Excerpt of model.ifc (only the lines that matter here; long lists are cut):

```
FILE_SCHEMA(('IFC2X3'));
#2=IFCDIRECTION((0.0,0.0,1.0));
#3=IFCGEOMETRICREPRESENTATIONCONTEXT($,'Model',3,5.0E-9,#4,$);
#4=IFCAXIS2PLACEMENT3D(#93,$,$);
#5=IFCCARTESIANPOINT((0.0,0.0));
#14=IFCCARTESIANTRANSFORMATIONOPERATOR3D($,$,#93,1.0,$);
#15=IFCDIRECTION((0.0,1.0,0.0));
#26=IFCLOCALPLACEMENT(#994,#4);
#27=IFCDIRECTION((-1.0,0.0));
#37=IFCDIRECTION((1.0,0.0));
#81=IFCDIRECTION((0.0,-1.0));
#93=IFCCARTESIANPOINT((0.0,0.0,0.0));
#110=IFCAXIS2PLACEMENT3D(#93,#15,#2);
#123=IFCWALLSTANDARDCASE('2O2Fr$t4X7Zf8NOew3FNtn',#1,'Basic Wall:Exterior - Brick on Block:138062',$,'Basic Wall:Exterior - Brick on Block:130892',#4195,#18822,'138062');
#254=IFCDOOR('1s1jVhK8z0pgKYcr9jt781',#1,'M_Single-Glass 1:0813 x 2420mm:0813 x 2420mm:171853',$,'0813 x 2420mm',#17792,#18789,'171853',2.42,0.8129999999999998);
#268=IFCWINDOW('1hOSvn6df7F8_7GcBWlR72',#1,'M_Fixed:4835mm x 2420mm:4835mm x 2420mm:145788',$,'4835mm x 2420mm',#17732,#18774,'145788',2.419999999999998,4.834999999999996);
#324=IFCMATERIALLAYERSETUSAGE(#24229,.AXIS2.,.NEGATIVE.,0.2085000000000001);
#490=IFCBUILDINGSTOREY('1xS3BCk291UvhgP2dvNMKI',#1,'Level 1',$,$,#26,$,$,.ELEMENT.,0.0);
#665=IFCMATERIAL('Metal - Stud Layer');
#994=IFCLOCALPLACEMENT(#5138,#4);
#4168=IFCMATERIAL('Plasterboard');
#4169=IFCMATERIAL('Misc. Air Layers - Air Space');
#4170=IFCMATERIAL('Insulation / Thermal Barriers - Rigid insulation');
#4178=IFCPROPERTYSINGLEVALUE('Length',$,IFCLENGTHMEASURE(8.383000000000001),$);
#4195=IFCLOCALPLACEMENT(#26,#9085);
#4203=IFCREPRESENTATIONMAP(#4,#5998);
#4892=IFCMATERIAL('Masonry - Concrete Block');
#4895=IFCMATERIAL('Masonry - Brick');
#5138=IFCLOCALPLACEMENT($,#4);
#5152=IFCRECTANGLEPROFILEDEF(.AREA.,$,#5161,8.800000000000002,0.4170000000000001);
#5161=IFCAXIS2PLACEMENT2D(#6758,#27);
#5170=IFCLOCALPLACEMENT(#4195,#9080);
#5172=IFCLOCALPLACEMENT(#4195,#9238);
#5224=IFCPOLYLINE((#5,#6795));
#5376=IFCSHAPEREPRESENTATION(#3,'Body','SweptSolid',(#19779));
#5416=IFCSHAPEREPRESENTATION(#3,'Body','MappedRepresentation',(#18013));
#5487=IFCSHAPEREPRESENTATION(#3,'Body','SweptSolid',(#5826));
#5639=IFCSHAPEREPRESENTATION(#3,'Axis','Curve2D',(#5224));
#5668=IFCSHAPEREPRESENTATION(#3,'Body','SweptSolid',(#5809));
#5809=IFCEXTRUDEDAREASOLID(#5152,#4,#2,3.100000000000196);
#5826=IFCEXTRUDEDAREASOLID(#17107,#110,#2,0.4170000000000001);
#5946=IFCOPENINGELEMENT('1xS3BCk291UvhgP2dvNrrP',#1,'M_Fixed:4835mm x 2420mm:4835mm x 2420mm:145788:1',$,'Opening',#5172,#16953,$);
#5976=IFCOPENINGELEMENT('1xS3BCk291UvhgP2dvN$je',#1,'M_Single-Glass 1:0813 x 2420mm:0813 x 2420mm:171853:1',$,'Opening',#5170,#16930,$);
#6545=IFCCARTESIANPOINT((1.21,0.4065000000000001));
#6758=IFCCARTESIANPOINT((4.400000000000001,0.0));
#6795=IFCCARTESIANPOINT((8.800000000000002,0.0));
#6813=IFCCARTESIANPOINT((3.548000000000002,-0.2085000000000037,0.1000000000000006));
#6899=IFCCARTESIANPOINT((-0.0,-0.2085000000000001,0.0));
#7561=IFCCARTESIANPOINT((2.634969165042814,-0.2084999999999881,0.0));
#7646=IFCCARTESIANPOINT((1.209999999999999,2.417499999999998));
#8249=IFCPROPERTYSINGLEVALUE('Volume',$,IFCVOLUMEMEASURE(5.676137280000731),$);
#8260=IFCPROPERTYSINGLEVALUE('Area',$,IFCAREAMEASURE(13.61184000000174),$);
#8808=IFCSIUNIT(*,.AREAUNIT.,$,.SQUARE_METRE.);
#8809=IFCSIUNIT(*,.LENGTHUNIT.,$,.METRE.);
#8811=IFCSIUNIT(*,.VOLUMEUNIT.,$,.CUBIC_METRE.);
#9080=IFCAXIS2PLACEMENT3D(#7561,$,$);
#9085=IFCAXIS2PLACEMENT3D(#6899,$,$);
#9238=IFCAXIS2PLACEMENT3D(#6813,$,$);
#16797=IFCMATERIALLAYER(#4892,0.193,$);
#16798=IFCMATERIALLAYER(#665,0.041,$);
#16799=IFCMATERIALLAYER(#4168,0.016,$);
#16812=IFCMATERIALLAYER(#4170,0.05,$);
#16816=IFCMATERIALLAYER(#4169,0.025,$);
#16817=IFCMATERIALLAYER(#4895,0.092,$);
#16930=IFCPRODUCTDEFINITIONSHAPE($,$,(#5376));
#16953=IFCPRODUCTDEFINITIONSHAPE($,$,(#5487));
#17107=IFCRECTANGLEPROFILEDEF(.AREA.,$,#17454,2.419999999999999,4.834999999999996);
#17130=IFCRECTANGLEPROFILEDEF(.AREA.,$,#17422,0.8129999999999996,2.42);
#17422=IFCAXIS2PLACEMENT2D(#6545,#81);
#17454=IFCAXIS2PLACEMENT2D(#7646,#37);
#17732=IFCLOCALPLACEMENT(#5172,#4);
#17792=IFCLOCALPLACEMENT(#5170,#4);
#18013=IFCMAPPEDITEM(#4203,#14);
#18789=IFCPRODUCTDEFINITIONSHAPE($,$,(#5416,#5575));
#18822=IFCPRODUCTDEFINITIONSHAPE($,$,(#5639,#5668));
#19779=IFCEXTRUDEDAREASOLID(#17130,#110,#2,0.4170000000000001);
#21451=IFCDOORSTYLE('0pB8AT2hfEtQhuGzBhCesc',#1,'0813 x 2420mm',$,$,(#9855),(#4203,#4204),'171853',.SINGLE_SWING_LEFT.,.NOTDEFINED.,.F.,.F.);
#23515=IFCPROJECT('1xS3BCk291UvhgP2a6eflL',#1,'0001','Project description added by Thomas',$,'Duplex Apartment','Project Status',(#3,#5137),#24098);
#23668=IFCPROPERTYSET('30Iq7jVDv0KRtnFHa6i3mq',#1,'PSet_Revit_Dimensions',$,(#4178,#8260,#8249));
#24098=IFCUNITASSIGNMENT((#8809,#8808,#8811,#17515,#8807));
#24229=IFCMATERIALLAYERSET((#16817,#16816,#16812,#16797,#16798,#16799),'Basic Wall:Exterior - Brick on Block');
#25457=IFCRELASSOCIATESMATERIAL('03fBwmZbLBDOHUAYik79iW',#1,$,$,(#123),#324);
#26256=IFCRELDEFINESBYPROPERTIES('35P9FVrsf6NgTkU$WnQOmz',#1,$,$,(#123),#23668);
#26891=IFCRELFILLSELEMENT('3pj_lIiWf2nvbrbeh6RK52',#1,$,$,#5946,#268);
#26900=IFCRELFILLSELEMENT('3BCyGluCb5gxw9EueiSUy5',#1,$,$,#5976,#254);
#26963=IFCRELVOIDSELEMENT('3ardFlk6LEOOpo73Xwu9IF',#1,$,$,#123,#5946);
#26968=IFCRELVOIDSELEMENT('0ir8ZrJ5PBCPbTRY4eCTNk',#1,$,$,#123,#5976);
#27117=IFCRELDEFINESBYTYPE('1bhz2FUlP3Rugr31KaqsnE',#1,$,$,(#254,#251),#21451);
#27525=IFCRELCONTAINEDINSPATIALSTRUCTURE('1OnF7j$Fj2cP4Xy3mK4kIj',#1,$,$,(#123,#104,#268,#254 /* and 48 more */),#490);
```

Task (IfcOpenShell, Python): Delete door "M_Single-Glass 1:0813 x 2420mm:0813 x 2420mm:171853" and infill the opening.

```python
import ifcopenshell
import ifcopenshell.api.feature
import ifcopenshell.api.pset
import ifcopenshell.api.root
import ifcopenshell.geom
import ifcopenshell.util.element
import ifcopenshell.util.shape
import ifcopenshell.util.unit

model = ifcopenshell.open("model.ifc")
area_scale = ifcopenshell.util.unit.calculate_unit_scale(model, "AREAUNIT")
volume_scale = ifcopenshell.util.unit.calculate_unit_scale(model, "VOLUMEUNIT")
settings = ifcopenshell.geom.settings()


def volume(element):
    """Net volume in cubic metres, openings subtracted."""
    shape = ifcopenshell.geom.create_shape(settings, element)
    return ifcopenshell.util.shape.get_volume(shape.geometry)


door = model.by_id(254)
opening = door.FillsVoids[0].RelatingOpeningElement
wall = opening.VoidsElements[0].RelatingBuildingElement
before = volume(wall)

ifcopenshell.api.root.remove_product(model, product=door)
ifcopenshell.api.feature.remove_feature(model, feature=opening)

after = volume(wall)
thickness = 0.417  # wall thickness in metres

# Update the wall's stored quantities.
pset = model.by_id(ifcopenshell.util.element.get_pset(wall, "PSet_Revit_Dimensions", should_inherit=False)["id"])
ifcopenshell.api.pset.edit_pset(model, pset=pset, properties={
    "Area": model.create_entity("IfcAreaMeasure", after / thickness / area_scale),
    "Volume": model.create_entity("IfcVolumeMeasure", after / volume_scale),
})

print(f"wall volume {before:.3f} -> {after:.3f} m3")

model.write("model_edited.ifc")
```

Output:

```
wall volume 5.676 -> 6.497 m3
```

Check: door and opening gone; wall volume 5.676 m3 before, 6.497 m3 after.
